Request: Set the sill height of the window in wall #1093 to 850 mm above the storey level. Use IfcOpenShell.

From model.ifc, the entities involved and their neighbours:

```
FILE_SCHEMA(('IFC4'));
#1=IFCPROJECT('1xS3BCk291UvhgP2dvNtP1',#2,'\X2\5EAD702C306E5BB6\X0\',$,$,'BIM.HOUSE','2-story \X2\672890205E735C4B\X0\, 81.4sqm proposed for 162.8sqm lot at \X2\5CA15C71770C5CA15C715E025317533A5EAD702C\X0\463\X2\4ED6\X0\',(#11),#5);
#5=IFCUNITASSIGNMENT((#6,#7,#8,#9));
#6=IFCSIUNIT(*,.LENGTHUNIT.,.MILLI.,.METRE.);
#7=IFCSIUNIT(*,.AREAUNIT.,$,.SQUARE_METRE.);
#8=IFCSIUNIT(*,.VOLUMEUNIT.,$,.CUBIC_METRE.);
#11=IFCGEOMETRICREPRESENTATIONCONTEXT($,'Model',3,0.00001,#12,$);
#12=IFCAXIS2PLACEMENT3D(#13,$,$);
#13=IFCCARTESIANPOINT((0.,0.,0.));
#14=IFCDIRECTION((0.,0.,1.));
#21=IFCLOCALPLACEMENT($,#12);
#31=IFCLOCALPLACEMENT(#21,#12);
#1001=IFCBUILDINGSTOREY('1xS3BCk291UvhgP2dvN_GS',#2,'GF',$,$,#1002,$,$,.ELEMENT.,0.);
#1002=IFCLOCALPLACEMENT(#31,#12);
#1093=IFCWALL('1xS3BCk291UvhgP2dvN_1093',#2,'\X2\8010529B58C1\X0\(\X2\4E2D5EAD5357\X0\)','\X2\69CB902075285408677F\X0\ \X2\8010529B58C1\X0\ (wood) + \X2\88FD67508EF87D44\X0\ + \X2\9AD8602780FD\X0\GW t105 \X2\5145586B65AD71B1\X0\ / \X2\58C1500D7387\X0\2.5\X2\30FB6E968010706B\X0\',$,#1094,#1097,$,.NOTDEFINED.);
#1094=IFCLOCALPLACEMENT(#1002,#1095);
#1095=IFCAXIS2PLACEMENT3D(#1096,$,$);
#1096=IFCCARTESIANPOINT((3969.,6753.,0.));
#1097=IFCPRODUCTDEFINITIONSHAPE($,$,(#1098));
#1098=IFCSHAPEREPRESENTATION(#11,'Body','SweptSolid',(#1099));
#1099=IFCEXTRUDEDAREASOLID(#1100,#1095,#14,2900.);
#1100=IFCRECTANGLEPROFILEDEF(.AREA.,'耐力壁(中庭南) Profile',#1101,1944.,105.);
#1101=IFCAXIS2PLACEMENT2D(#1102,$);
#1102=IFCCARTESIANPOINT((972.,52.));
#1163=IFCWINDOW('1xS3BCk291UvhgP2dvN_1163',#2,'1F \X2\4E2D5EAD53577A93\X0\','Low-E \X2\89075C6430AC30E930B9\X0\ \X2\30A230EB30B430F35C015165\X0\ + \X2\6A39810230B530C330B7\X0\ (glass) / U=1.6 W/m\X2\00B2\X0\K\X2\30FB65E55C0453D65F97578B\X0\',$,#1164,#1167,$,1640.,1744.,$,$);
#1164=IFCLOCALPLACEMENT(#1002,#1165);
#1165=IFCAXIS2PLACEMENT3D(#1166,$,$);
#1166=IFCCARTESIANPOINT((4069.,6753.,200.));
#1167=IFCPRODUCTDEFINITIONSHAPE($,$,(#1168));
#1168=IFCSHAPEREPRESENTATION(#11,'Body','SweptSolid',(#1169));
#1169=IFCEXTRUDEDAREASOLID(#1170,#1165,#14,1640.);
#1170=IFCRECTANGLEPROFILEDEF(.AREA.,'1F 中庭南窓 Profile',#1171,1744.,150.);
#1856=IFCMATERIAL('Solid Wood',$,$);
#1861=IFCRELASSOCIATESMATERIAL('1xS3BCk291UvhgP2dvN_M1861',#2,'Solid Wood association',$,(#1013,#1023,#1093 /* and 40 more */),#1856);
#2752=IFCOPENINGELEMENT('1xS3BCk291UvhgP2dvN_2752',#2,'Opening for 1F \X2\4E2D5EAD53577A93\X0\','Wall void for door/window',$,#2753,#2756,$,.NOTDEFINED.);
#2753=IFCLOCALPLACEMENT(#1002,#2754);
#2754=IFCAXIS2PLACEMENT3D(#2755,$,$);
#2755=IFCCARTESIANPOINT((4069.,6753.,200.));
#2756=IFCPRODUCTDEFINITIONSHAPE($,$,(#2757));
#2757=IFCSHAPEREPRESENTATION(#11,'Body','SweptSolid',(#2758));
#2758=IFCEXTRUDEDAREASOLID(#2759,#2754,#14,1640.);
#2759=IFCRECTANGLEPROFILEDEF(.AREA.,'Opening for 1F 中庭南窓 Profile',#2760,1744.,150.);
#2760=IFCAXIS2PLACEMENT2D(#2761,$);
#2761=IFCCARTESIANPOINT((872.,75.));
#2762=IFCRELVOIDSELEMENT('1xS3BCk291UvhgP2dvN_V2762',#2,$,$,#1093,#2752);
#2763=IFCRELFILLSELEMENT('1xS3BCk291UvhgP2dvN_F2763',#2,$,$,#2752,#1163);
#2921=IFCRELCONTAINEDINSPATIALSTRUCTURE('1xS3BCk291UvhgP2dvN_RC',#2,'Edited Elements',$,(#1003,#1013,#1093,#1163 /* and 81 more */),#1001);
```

```python
import numpy as np
import ifcopenshell
import ifcopenshell.api.geometry
import ifcopenshell.geom
import ifcopenshell.util.element
import ifcopenshell.util.placement
import ifcopenshell.util.shape
import ifcopenshell.util.unit

model = ifcopenshell.open("model.ifc")
unit_scale = ifcopenshell.util.unit.calculate_unit_scale(model)

window = model.by_guid("1xS3BCk291UvhgP2dvN_1163")
opening = window.FillsVoids[0].RelatingOpeningElement
storey = ifcopenshell.util.element.get_container(window, ifc_class="IfcBuildingStorey")
level = ifcopenshell.util.placement.get_local_placement(storey.ObjectPlacement)[2, 3]

# The opening's origin need not be at the sill, so measure its lowest point.
shape = ifcopenshell.geom.create_shape(ifcopenshell.geom.settings(), opening)
bottom = ifcopenshell.util.shape.get_shape_bottom_elevation(shape, shape.geometry) / unit_scale
dz = level + 0.85 / unit_scale - bottom

shift = np.array([0.0, 0.0, dz])
# The window is not placed relative to its opening, so move both.
for product in (opening, window):
    matrix = ifcopenshell.util.placement.get_local_placement(product.ObjectPlacement)
    matrix[:3, 3] += shift
    ifcopenshell.api.geometry.edit_object_placement(model, product=product, matrix=matrix, is_si=False)

print(f"moved by {dz * unit_scale:+.3f} m")

model.write("model_edited.ifc")
```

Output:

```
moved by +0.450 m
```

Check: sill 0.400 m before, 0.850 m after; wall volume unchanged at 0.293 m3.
